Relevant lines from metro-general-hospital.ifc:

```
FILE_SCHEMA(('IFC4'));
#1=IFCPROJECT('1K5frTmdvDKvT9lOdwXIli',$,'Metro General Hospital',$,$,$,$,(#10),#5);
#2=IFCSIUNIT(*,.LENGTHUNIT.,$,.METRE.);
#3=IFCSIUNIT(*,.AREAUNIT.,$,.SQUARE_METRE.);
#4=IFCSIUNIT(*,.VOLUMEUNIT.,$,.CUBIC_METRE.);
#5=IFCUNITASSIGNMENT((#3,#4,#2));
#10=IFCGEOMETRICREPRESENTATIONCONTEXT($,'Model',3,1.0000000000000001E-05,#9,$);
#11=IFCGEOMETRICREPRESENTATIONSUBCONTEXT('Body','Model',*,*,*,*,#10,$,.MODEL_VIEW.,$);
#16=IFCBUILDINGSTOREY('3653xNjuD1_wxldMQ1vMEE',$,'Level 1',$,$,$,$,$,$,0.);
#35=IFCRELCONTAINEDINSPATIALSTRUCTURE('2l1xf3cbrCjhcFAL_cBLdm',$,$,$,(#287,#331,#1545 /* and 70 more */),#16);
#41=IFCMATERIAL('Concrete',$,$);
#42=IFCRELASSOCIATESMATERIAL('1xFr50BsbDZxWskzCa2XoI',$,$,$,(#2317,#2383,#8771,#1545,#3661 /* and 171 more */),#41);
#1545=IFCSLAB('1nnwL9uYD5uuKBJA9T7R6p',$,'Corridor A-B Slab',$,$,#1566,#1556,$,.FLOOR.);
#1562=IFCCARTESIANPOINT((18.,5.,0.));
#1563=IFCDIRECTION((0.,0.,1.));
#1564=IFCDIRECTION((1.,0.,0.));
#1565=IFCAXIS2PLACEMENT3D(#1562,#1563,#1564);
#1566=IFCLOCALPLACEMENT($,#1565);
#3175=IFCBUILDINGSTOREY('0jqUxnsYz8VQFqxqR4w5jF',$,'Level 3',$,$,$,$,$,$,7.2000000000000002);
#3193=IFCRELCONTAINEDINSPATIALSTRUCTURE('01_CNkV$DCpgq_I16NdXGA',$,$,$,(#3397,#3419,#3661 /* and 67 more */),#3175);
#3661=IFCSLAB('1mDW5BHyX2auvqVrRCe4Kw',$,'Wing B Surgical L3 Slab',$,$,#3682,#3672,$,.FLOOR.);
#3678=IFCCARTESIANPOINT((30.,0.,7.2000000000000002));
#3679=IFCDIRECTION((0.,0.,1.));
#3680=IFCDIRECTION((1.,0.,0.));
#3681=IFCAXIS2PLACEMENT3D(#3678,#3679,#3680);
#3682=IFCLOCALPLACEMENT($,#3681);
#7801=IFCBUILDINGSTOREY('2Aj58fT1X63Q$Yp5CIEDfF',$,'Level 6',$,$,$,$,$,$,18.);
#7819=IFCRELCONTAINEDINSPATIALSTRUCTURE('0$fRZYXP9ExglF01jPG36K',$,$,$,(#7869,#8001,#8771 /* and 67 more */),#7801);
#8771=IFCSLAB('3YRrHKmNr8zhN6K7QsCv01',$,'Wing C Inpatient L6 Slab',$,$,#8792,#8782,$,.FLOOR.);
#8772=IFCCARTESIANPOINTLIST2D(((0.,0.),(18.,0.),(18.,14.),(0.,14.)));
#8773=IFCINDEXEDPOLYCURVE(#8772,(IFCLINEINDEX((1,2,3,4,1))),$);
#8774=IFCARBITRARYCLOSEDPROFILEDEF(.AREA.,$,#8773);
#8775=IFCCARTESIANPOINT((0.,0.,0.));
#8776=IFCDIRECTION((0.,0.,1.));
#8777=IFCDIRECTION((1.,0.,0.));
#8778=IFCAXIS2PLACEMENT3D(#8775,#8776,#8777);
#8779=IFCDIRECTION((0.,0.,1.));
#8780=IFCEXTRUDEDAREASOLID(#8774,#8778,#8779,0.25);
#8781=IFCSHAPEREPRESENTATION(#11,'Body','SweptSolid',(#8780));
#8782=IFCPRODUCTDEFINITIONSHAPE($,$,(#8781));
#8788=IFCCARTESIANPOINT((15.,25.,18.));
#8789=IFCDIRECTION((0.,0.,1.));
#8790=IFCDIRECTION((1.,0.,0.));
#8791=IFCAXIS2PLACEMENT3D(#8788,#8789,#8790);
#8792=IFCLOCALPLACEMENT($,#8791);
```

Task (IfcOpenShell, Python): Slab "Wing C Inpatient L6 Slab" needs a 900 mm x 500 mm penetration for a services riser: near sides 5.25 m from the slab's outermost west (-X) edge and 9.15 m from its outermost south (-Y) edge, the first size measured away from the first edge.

```python
import numpy as np
import ifcopenshell
import ifcopenshell.api.feature
import ifcopenshell.api.geometry
import ifcopenshell.api.root
import ifcopenshell.geom
import ifcopenshell.util.placement
import ifcopenshell.util.representation
import ifcopenshell.util.shape
import ifcopenshell.util.unit

model = ifcopenshell.open("metro-general-hospital.ifc")
unit_scale = ifcopenshell.util.unit.calculate_unit_scale(model)
settings = ifcopenshell.geom.settings()


def volume(element):
    """Net volume in cubic metres, openings subtracted."""
    shape = ifcopenshell.geom.create_shape(settings, element)
    return ifcopenshell.util.shape.get_volume(shape.geometry)


slab = model.by_guid("3YRrHKmNr8zhN6K7QsCv01")
before = volume(slab)

# Extent in the slab's own axes, in metres. The edges named are its -X and -Y sides.
slab_shape = ifcopenshell.geom.create_shape(settings, slab)
vertices = ifcopenshell.util.shape.get_vertices(slab_shape.geometry)
x_min, y_min, bottom = vertices.min(axis=0)
top = vertices[:, 2].max()

opening = ifcopenshell.api.root.create_entity(model, ifc_class="IfcOpeningElement", name="Services riser opening", predefined_type="OPENING")
context = ifcopenshell.util.representation.get_context(model, "Model", "Body", "MODEL_VIEW")
width, depth = 0.9, 0.5
outline = [(0.0, 0.0), (width, 0.0), (width, depth), (0.0, depth), (0.0, 0.0)]
# Overshoot both faces by 50 mm so the cut is clean.
shape = ifcopenshell.api.geometry.add_slab_representation(
    model, context=context, depth=top - bottom + 0.1, polyline=outline
)
ifcopenshell.api.geometry.assign_representation(model, product=opening, representation=shape)

matrix = ifcopenshell.util.placement.get_local_placement(slab.ObjectPlacement)
matrix[:, 3] = matrix @ np.append(np.array([x_min + 5.25, y_min + 9.15, bottom - 0.05]) / unit_scale, 1.0)
ifcopenshell.api.geometry.edit_object_placement(model, product=opening, matrix=matrix, is_si=False)
ifcopenshell.api.feature.add_feature(model, feature=opening, element=slab)

after = volume(slab)

print(f"slab volume {before:.3f} -> {after:.3f} m3")

model.write("metro-general-hospital_edited.ifc")
```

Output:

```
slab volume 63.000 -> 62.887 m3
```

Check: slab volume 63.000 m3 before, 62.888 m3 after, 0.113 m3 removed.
